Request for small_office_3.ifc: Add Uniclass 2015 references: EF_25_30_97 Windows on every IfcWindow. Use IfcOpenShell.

First a look at what the model holds.

```python
import ifcopenshell

model = ifcopenshell.open("small_office_3.ifc")
print(model.schema)
print("classifications:", [c.Name for c in model.by_type("IfcClassification")])
for ifc_class in ("IfcDoor", "IfcRoof", "IfcStair", "IfcWall", "IfcWindow"):
    print(ifc_class, len(model.by_type(ifc_class)))
```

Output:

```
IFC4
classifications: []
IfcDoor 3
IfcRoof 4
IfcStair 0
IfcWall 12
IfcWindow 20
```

```python
import ifcopenshell
import ifcopenshell.api.classification

model = ifcopenshell.open("small_office_3.ifc")

system = ifcopenshell.api.classification.add_classification(model, classification="Uniclass 2015")

codes = {
    "IfcWindow": ("EF_25_30_97", "Windows"),
}
for ifc_class, (code, name) in codes.items():
    products = model.by_type(ifc_class)
    ifcopenshell.api.classification.add_reference(
        model, products=products, classification=system, identification=code, name=name
    )
    print(code, len(products))

model.write("small_office_3_rev.ifc")
```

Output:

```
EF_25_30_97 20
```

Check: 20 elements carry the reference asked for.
